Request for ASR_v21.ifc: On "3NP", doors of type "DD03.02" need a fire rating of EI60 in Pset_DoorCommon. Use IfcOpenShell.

First a look at what the model holds.

```python
import ifcopenshell
import ifcopenshell.util.element

model = ifcopenshell.open("ASR_v21.ifc")
print(model.schema)
storey = next(s for s in model.by_type("IfcBuildingStorey") if s.Name == "3NP")
doors = [e for e in ifcopenshell.util.element.get_decomposition(storey) if e.is_a("IfcDoor")]
seen = {}
for e in doors:
    element_type = ifcopenshell.util.element.get_type(e)
    key = (element_type.Name if element_type != e and element_type else None, ifcopenshell.util.element.get_pset(e, "Pset_DoorCommon", "FireRating"))
    seen[key] = seen.get(key, 0) + 1
for (name, value), count in sorted(seen.items(), key=str):
    print(count, "x", name, "|", value)
```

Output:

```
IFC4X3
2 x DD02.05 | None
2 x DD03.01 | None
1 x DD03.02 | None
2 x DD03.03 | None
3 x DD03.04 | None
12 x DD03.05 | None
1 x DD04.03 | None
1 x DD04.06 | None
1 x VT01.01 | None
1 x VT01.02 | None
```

```python
import ifcopenshell
import ifcopenshell.api.pset
import ifcopenshell.util.element

model = ifcopenshell.open("ASR_v21.ifc")

storey = next(s for s in model.by_type("IfcBuildingStorey") if s.Name == "3NP")
doors = [e for e in ifcopenshell.util.element.get_decomposition(storey) if e.is_a("IfcDoor")]

count = 0
for e in doors:
    element_type = ifcopenshell.util.element.get_type(e)
    if element_type in (None, e) or element_type.Name != "DD03.02":
        continue
    # add_pset returns the element's existing set when there is one.
    pset = ifcopenshell.api.pset.add_pset(model, product=e, name="Pset_DoorCommon")
    ifcopenshell.api.pset.edit_pset(model, pset=pset, properties={"FireRating": "EI60"})
    count += 1

print(count, "doors updated")

model.write("ASR_v21_v2.ifc")
```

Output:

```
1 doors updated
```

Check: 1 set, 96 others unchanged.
